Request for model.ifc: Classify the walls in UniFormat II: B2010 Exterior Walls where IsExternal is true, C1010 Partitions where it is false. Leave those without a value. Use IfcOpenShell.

First a look at what the model holds.

```python
import ifcopenshell
import ifcopenshell.util.element

model = ifcopenshell.open("model.ifc")
print(model.schema)
print("classifications:", [c.Name for c in model.by_type("IfcClassification")])
values = [ifcopenshell.util.element.get_pset(e, "Pset_WallCommon", "IsExternal") for e in model.by_type("IfcWall")]
for value in (True, False, None):
    print("IsExternal", value, values.count(value))
```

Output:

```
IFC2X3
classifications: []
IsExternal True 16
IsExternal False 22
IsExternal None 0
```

```python
import ifcopenshell
import ifcopenshell.api.classification
import ifcopenshell.util.element

model = ifcopenshell.open("model.ifc")

# IFC2X3 requires Source and Edition and has no link from the project to the system.
system = model.create_entity("IfcClassification", Source="ASTM", Edition="E1557", Name="UniFormat II")

walls = model.by_type("IfcWall")
external = {e: ifcopenshell.util.element.get_pset(e, "Pset_WallCommon", "IsExternal") for e in walls}
for flag, code, name in ((True, "B2010", "Exterior Walls"), (False, "C1010", "Partitions")):
    products = [e for e in walls if external[e] is flag]
    ifcopenshell.api.classification.add_reference(
        model, products=products, classification=system, identification=code, name=name
    )
    print(code, len(products))

model.write("model_edited.ifc")
```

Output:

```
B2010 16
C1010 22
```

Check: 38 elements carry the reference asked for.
